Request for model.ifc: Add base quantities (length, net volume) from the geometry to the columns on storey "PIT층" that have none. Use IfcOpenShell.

First a look at what the model holds.

```python
import ifcopenshell
import ifcopenshell.util.element
import ifcopenshell.util.unit

model = ifcopenshell.open("model.ifc")
print(model.schema)
for unit_type in ("LENGTHUNIT", "AREAUNIT", "VOLUMEUNIT"):
    print(unit_type, ifcopenshell.util.unit.calculate_unit_scale(model, unit_type))
storey = next(s for s in model.by_type("IfcBuildingStorey") if s.Name == "PIT층")
columns = [e for e in ifcopenshell.util.element.get_decomposition(storey) if e.is_a("IfcColumn")]
for e in sorted(columns, key=lambda e: e.id()):
    print(e.id(), e.is_a(), e.Name, list(ifcopenshell.util.element.get_psets(e, qtos_only=True)), sep=" | ")
```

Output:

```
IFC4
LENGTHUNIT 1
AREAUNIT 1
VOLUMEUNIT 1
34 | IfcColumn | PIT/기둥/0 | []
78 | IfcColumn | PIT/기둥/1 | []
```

```python
import ifcopenshell
import ifcopenshell.api.pset
import ifcopenshell.geom
import ifcopenshell.util.element
import ifcopenshell.util.shape
import ifcopenshell.util.unit

model = ifcopenshell.open("model.ifc")
unit_scale = ifcopenshell.util.unit.calculate_unit_scale(model)
volume_scale = ifcopenshell.util.unit.calculate_unit_scale(model, "VOLUMEUNIT")
settings = ifcopenshell.geom.settings()

storey = next(s for s in model.by_type("IfcBuildingStorey") if s.Name == "PIT층")
columns = [e for e in ifcopenshell.util.element.get_decomposition(storey) if e.is_a("IfcColumn")]

for e in sorted(columns, key=lambda e: e.id()):
    if ifcopenshell.util.element.get_psets(e, qtos_only=True, should_inherit=False):
        continue
    # Geometry comes back in metres, in the element's own axes.
    shape = ifcopenshell.geom.create_shape(settings, e)
    values = {
        "Length": ifcopenshell.util.shape.get_z(shape.geometry) / unit_scale,
        "NetVolume": ifcopenshell.util.shape.get_volume(shape.geometry) / volume_scale,
    }
    qto = ifcopenshell.api.pset.add_qto(model, product=e, name="Qto_ColumnBaseQuantities")
    ifcopenshell.api.pset.edit_qto(model, qto=qto, properties=values)
    print(e.id(), {k: round(v, 3) for k, v in values.items()})

model.write("model_rev.ifc")
```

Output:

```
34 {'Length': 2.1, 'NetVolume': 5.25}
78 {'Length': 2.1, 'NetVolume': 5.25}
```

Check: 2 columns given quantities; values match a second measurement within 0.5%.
